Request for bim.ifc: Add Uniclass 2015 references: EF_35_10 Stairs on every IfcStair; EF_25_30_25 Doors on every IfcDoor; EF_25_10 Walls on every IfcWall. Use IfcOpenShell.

First a look at what the model holds.

```python
import ifcopenshell

model = ifcopenshell.open("bim.ifc")
print(model.schema)
print("classifications:", [c.Name for c in model.by_type("IfcClassification")])
for ifc_class in ("IfcDoor", "IfcRoof", "IfcStair", "IfcWall", "IfcWindow"):
    print(ifc_class, len(model.by_type(ifc_class)))
```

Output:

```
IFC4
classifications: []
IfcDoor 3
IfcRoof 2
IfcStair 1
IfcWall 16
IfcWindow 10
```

```python
import ifcopenshell
import ifcopenshell.api.classification

model = ifcopenshell.open("bim.ifc")

system = ifcopenshell.api.classification.add_classification(model, classification="Uniclass 2015")

codes = {
    "IfcStair": ("EF_35_10", "Stairs"),
    "IfcDoor": ("EF_25_30_25", "Doors"),
    "IfcWall": ("EF_25_10", "Walls"),
}
for ifc_class, (code, name) in codes.items():
    products = model.by_type(ifc_class)
    ifcopenshell.api.classification.add_reference(
        model, products=products, classification=system, identification=code, name=name
    )
    print(code, len(products))

model.write("bim_edited.ifc")
```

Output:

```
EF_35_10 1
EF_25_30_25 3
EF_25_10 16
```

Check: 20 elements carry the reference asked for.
